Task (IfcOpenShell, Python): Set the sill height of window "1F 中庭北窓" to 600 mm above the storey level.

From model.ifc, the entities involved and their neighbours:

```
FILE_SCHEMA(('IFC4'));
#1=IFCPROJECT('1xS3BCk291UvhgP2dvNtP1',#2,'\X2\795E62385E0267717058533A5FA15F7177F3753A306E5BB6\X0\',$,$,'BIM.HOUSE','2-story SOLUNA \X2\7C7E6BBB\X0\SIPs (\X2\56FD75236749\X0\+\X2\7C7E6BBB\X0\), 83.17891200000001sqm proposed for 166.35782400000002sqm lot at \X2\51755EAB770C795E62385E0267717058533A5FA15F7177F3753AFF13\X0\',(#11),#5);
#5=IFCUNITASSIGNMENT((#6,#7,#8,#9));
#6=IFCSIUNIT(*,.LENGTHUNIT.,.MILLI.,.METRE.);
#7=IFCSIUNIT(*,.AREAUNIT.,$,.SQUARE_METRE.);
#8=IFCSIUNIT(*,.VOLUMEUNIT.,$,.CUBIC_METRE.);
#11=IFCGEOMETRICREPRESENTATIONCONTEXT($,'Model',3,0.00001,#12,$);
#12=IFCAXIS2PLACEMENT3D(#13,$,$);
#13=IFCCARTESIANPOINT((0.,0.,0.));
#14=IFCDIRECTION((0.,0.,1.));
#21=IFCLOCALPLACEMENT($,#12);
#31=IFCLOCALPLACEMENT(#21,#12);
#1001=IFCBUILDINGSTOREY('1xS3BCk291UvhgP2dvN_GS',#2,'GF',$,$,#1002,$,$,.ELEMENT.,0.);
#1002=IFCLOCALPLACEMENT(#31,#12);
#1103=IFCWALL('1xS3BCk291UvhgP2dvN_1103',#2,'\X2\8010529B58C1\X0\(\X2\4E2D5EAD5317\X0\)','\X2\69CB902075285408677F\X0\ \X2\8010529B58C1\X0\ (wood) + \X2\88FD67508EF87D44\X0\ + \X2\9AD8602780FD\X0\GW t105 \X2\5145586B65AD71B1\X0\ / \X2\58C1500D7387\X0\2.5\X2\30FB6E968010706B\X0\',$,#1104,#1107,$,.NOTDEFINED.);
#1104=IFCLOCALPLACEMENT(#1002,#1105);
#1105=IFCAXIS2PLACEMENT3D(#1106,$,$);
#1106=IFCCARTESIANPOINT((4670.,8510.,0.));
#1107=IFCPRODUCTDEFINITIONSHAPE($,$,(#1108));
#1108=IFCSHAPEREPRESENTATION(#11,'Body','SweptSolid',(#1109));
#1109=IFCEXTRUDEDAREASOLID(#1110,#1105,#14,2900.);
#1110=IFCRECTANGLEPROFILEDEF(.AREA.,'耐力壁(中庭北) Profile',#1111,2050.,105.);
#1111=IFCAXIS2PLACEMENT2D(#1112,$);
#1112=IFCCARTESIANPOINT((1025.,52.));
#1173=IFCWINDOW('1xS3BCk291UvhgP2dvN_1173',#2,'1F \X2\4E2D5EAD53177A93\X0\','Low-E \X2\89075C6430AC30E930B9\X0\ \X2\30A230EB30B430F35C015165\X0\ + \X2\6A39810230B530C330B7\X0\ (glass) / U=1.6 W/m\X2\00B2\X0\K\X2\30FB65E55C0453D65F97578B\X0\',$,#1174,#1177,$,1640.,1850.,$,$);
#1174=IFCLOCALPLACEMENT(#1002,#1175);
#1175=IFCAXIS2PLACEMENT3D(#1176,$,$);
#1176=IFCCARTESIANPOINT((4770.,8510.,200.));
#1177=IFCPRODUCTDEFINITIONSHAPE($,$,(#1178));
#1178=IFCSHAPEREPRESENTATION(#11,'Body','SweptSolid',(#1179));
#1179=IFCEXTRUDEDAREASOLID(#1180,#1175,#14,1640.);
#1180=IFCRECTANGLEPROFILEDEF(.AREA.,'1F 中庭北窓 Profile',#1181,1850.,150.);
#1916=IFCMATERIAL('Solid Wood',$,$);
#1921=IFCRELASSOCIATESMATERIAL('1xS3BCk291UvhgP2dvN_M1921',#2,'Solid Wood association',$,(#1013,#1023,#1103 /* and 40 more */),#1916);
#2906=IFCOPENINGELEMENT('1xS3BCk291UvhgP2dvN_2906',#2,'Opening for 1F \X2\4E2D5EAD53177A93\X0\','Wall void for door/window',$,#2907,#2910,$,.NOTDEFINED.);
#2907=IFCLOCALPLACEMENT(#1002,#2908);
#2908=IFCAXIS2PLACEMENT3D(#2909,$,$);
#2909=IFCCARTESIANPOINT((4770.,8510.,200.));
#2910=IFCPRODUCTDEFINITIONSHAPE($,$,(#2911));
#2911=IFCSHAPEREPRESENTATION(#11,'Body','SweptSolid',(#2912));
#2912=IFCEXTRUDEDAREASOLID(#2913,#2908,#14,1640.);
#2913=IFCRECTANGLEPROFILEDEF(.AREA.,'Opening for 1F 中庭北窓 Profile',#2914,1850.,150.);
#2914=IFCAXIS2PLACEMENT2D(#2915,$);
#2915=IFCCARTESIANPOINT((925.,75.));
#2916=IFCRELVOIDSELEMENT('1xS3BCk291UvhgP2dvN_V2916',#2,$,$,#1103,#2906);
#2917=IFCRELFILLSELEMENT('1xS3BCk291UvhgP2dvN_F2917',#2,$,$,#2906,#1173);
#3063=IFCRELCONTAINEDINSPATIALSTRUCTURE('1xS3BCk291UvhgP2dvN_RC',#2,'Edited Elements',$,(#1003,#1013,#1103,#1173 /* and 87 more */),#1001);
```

```python
import numpy as np
import ifcopenshell
import ifcopenshell.api.geometry
import ifcopenshell.geom
import ifcopenshell.util.element
import ifcopenshell.util.placement
import ifcopenshell.util.shape
import ifcopenshell.util.unit

model = ifcopenshell.open("model.ifc")
unit_scale = ifcopenshell.util.unit.calculate_unit_scale(model)

window = model.by_guid("1xS3BCk291UvhgP2dvN_1173")
opening = window.FillsVoids[0].RelatingOpeningElement
storey = ifcopenshell.util.element.get_container(window, ifc_class="IfcBuildingStorey")
level = ifcopenshell.util.placement.get_local_placement(storey.ObjectPlacement)[2, 3]

# The opening's origin need not be at the sill, so measure its lowest point.
shape = ifcopenshell.geom.create_shape(ifcopenshell.geom.settings(), opening)
bottom = ifcopenshell.util.shape.get_shape_bottom_elevation(shape, shape.geometry) / unit_scale
dz = level + 600.0 - bottom

shift = np.array([0.0, 0.0, dz])
# The window is not placed relative to its opening, so move both.
for product in (opening, window):
    matrix = ifcopenshell.util.placement.get_local_placement(product.ObjectPlacement)
    matrix[:3, 3] += shift
    ifcopenshell.api.geometry.edit_object_placement(model, product=product, matrix=matrix, is_si=False)

print(f"moved by {dz * unit_scale:+.3f} m")

model.write("model_edited.ifc")
```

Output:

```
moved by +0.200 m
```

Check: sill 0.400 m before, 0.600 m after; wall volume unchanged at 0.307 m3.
